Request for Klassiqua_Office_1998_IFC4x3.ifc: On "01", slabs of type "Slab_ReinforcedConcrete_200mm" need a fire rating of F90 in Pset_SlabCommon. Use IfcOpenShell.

First a look at what the model holds.

```python
import ifcopenshell
import ifcopenshell.util.element

model = ifcopenshell.open("Klassiqua_Office_1998_IFC4x3.ifc")
print(model.schema)
storey = next(s for s in model.by_type("IfcBuildingStorey") if s.Name == "01")
slabs = [e for e in ifcopenshell.util.element.get_decomposition(storey) if e.is_a("IfcSlab")]
seen = {}
for e in slabs:
    element_type = ifcopenshell.util.element.get_type(e)
    key = (element_type.Name if element_type != e and element_type else None, ifcopenshell.util.element.get_pset(e, "Pset_SlabCommon", "FireRating"))
    seen[key] = seen.get(key, 0) + 1
for (name, value), count in sorted(seen.items(), key=str):
    print(count, "x", name, "|", value)
```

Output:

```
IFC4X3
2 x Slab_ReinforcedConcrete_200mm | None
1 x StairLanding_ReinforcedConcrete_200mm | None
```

```python
import ifcopenshell
import ifcopenshell.api.pset
import ifcopenshell.util.element

model = ifcopenshell.open("Klassiqua_Office_1998_IFC4x3.ifc")

storey = next(s for s in model.by_type("IfcBuildingStorey") if s.Name == "01")
slabs = [e for e in ifcopenshell.util.element.get_decomposition(storey) if e.is_a("IfcSlab")]

count = 0
for e in slabs:
    element_type = ifcopenshell.util.element.get_type(e)
    if element_type in (None, e) or element_type.Name != "Slab_ReinforcedConcrete_200mm":
        continue
    # add_pset returns the element's existing set when there is one.
    pset = ifcopenshell.api.pset.add_pset(model, product=e, name="Pset_SlabCommon")
    ifcopenshell.api.pset.edit_pset(model, pset=pset, properties={"FireRating": "F90"})
    count += 1

print(count, "slabs updated")

model.write("Klassiqua_Office_1998_IFC4x3_rev.ifc")
```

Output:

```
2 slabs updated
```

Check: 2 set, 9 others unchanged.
